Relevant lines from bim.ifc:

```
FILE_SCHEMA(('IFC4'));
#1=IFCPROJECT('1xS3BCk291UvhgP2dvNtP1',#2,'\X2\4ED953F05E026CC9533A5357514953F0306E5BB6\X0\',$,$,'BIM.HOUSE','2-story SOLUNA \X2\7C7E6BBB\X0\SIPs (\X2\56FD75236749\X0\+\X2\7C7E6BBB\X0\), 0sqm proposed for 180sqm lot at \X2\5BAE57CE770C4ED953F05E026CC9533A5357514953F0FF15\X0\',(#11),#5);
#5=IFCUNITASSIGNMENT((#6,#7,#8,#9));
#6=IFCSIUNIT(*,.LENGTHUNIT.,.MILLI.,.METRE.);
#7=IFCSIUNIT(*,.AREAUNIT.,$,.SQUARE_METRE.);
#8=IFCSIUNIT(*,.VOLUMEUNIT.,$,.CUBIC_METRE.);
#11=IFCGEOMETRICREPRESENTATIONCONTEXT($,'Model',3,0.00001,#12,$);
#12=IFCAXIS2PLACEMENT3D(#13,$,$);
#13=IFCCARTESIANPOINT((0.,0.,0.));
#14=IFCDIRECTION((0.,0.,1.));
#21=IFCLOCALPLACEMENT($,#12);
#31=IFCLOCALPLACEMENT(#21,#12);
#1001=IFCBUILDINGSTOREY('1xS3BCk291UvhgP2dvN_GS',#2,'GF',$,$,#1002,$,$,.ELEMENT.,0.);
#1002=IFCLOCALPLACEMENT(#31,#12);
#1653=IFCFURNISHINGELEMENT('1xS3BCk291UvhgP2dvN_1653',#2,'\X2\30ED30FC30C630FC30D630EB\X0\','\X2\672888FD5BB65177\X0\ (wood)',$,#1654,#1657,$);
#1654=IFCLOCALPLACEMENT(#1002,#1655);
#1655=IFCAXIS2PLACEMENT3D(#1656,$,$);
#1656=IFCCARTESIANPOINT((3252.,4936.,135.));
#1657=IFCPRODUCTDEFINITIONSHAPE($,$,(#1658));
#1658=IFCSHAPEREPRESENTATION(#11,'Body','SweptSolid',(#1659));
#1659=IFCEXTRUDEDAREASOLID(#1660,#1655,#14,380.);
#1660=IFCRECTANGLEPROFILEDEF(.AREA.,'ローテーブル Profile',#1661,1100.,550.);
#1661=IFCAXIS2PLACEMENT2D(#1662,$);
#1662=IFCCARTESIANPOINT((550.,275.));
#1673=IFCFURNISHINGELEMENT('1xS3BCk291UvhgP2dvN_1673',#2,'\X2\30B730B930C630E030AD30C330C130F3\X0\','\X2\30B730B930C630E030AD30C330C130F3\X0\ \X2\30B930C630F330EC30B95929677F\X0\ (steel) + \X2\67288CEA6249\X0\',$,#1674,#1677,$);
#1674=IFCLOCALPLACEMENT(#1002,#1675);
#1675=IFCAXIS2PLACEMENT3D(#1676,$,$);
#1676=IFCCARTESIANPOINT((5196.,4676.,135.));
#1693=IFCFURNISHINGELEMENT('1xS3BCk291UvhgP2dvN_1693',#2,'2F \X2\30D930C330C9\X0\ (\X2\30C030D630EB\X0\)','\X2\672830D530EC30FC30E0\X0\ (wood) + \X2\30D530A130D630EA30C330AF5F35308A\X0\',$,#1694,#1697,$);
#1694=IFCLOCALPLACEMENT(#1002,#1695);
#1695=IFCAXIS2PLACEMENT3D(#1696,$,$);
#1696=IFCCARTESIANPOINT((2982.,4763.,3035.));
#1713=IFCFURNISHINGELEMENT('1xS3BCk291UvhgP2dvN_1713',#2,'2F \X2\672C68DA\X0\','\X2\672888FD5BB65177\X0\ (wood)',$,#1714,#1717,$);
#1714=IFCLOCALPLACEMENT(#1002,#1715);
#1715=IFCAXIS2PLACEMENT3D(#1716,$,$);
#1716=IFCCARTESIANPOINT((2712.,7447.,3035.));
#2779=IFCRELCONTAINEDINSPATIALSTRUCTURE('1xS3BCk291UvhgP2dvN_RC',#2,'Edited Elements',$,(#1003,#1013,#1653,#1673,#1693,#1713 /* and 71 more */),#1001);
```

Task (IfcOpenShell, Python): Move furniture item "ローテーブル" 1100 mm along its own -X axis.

```python
import ifcopenshell
import ifcopenshell.api.geometry
import ifcopenshell.util.placement

model = ifcopenshell.open("bim.ifc")

item = model.by_guid("1xS3BCk291UvhgP2dvN_1653")
matrix = ifcopenshell.util.placement.get_local_placement(item.ObjectPlacement)
matrix[:3, 3] -= matrix[:3, 0] * 1100.0
ifcopenshell.api.geometry.edit_object_placement(model, product=item, matrix=matrix, is_si=False)

print(ifcopenshell.util.placement.get_local_placement(item.ObjectPlacement).round(3) + 0.0)

model.write("bim-out.ifc")
```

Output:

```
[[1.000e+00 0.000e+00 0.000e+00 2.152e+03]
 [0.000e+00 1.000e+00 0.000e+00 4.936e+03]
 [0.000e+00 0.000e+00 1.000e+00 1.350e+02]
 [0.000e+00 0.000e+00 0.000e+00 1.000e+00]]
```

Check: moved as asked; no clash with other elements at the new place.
